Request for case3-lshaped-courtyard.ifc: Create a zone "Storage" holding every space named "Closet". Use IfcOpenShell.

First a look at what the model holds.

```python
import ifcopenshell

model = ifcopenshell.open("case3-lshaped-courtyard.ifc")
print(model.schema)
seen = {}
for space in model.by_type("IfcSpace"):
    seen[space.Name] = seen.get(space.Name, 0) + 1
for name, count in sorted(seen.items(), key=str):
    print(count, "x", name)
print("zones:", [z.Name for z in model.by_type("IfcZone")][:20])
```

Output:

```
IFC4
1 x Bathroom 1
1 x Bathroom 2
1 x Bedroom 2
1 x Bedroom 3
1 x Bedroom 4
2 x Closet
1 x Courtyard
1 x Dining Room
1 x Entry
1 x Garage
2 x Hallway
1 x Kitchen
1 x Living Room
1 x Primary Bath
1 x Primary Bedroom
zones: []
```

```python
import ifcopenshell
import ifcopenshell.api.group
import ifcopenshell.api.root

model = ifcopenshell.open("case3-lshaped-courtyard.ifc")

names = {"Closet"}
spaces = [s for s in model.by_type("IfcSpace") if s.Name in names]

zone = ifcopenshell.api.root.create_entity(model, ifc_class="IfcZone", name="Storage")
ifcopenshell.api.group.assign_group(model, products=spaces, group=zone)
print(len(spaces), "spaces in", zone.Name)

model.write("case3-lshaped-courtyard_updated.ifc")
```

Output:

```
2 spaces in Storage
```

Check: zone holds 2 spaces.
